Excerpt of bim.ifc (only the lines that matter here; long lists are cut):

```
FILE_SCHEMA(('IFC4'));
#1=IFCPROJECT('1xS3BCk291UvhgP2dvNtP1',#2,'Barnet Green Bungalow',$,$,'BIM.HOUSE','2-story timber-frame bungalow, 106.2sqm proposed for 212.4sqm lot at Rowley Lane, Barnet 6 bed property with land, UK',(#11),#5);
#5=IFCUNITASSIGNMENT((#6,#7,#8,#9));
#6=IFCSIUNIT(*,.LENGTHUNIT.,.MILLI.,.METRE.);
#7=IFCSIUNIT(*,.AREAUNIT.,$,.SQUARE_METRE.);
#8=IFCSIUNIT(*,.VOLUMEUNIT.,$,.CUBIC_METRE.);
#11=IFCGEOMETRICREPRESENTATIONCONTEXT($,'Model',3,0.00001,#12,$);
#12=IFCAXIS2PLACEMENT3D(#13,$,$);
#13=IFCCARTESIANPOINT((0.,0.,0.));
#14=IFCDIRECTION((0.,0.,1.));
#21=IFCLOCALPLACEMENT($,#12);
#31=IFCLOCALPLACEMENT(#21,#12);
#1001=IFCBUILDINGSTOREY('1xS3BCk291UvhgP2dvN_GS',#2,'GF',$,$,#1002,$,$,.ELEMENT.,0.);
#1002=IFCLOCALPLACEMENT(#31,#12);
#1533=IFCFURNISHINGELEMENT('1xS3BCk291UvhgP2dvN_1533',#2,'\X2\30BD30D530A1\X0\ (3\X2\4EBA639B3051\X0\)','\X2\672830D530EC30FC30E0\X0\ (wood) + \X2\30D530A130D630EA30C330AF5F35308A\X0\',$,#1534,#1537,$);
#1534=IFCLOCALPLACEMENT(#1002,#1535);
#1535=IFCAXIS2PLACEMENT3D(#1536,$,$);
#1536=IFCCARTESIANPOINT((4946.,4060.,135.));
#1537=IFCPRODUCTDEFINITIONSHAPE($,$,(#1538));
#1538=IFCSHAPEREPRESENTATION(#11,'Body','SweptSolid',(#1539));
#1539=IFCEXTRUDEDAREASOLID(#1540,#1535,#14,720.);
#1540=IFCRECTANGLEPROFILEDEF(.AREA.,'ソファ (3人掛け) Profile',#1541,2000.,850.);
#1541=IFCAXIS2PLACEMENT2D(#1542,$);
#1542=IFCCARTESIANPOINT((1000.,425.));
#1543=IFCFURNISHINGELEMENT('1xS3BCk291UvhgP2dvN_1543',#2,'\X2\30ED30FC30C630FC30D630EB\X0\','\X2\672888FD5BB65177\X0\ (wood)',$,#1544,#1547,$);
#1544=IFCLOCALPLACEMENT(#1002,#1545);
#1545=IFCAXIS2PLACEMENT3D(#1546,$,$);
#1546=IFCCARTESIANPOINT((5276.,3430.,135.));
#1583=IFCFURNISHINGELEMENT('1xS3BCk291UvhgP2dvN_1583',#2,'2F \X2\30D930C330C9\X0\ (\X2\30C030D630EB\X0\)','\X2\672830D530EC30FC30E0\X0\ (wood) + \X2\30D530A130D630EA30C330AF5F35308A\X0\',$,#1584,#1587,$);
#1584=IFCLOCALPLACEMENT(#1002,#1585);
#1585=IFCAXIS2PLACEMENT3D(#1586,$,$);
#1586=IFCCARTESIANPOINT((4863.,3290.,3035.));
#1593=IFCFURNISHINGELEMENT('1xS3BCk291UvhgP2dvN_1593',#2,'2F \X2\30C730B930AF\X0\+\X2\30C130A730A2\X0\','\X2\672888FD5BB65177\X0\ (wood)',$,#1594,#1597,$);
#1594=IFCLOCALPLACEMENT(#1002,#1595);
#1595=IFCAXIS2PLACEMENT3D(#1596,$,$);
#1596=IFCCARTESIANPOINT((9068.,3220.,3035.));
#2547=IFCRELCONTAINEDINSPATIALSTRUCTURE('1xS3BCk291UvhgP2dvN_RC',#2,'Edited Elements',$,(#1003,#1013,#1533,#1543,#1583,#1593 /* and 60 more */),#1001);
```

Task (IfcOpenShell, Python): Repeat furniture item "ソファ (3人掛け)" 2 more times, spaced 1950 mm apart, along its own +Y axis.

```python
import ifcopenshell
import ifcopenshell.api.geometry
import ifcopenshell.api.root
import ifcopenshell.util.element
import ifcopenshell.util.placement

model = ifcopenshell.open("bim.ifc")


def reuse_history(source, copy):
    """copy_class also copies each property set's owner history, people and application; keep the originals."""
    for rel in copy.IsDefinedBy:
        if rel.is_a("IfcRelDefinesByProperties") and (history := rel.RelatingPropertyDefinition.OwnerHistory):
            rel.RelatingPropertyDefinition.OwnerHistory = source.OwnerHistory
            ifcopenshell.util.element.remove_deep2(model, history)


source = model.by_guid("1xS3BCk291UvhgP2dvN_1533")
base = ifcopenshell.util.placement.get_local_placement(source.ObjectPlacement)
step = base[:3, 1] * 1950.0

for i in range(1, 3):
    copy = ifcopenshell.api.root.copy_class(model, product=source)
    copy.Representation = ifcopenshell.util.element.copy_deep(
        model, source.Representation, exclude=["IfcGeometricRepresentationContext", "IfcRepresentationMap"]
    )
    reuse_history(source, copy)
    matrix = base.copy()
    matrix[:3, 3] += i * step
    print("added at", matrix[:3, 3].round(3) + 0.0)
    ifcopenshell.api.geometry.edit_object_placement(model, product=copy, matrix=matrix, is_si=False)

model.write("bim_updated.ifc")
```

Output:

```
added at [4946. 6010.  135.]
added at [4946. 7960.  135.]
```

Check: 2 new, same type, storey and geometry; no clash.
